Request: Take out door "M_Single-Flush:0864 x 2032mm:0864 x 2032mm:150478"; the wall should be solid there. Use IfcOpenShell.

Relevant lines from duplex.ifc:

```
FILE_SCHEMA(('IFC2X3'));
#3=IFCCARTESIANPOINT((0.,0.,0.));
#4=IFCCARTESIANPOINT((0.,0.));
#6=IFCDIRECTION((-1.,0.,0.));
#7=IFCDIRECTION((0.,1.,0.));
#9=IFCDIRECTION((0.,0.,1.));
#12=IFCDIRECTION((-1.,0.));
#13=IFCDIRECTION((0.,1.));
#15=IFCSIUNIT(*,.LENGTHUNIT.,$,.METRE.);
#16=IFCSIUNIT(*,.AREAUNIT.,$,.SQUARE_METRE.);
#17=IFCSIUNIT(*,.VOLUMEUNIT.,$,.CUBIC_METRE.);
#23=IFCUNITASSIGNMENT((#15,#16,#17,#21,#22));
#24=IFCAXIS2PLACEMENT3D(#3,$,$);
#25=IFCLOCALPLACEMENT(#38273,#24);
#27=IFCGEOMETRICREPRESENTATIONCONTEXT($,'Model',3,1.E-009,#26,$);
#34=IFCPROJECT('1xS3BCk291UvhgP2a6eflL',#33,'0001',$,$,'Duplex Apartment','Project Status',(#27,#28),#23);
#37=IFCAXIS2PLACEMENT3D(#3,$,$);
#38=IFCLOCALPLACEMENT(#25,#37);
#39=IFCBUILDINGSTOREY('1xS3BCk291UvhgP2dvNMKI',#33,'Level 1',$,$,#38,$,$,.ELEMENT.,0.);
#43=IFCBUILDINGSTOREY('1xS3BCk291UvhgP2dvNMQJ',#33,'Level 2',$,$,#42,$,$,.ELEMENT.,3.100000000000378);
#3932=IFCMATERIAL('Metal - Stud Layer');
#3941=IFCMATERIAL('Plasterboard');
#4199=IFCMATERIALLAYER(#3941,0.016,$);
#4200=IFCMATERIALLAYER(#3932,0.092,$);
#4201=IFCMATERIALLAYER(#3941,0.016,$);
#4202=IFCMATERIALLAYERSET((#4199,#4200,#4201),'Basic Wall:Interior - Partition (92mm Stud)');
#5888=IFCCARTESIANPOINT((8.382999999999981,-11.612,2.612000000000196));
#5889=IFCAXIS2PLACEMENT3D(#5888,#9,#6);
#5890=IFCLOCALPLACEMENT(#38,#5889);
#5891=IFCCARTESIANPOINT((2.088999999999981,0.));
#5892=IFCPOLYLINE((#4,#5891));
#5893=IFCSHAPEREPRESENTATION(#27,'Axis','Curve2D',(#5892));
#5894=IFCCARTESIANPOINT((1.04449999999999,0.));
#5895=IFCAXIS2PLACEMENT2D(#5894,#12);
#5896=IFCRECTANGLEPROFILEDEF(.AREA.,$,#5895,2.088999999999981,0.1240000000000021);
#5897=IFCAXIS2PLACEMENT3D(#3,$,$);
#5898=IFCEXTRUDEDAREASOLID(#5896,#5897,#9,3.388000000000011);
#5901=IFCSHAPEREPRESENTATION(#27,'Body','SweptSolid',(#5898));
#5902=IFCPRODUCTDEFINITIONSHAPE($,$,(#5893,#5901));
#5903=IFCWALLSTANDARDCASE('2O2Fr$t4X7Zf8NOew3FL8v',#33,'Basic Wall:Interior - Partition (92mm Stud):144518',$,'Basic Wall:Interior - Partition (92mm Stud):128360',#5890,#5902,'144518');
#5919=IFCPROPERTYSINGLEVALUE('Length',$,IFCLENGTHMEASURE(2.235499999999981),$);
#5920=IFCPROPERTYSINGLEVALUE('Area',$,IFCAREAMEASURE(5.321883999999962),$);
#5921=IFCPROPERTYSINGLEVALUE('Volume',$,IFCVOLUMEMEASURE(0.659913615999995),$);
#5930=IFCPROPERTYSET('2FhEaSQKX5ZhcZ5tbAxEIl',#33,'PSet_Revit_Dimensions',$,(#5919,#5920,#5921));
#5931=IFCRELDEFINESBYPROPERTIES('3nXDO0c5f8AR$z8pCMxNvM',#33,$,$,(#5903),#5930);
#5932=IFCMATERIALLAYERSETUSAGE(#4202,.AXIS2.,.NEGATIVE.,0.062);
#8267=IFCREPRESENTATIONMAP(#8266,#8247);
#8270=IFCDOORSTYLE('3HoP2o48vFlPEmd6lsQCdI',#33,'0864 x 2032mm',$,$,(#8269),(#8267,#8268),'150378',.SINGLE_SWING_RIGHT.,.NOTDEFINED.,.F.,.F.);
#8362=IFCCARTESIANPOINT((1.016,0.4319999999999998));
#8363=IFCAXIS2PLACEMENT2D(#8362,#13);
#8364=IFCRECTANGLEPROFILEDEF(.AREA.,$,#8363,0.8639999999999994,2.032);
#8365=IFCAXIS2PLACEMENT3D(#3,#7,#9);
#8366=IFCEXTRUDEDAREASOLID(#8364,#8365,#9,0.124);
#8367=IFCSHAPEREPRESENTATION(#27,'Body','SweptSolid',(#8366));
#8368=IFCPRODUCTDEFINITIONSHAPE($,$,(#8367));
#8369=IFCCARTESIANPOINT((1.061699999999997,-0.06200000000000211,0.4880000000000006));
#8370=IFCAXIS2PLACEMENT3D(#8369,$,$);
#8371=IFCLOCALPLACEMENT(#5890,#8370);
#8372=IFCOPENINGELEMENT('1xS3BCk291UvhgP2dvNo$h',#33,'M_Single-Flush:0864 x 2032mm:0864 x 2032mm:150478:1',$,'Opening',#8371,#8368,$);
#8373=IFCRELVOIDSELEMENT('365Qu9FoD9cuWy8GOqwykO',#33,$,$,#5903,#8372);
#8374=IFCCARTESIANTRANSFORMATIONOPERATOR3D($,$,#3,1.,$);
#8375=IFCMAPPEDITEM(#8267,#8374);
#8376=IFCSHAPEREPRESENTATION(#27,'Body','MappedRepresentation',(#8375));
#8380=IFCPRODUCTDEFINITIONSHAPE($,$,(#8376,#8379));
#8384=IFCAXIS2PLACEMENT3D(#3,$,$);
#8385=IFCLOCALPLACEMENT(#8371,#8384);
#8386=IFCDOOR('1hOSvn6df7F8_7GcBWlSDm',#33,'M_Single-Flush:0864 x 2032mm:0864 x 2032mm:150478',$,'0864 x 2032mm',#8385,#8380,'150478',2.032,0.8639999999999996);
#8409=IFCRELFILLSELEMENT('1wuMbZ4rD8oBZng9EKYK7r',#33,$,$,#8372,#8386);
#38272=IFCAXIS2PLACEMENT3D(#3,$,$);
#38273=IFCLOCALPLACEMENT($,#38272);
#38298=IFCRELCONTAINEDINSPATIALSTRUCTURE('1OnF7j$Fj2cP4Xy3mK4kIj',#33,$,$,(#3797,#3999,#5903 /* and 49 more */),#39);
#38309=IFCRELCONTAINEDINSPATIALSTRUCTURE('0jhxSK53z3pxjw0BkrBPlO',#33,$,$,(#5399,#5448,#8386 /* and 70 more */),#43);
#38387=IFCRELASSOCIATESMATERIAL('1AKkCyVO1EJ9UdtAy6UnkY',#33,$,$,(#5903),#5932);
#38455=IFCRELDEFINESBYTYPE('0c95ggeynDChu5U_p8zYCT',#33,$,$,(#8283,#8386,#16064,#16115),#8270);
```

```python
import ifcopenshell
import ifcopenshell.api.feature
import ifcopenshell.api.pset
import ifcopenshell.api.root
import ifcopenshell.geom
import ifcopenshell.util.element
import ifcopenshell.util.shape
import ifcopenshell.util.unit

model = ifcopenshell.open("duplex.ifc")
area_scale = ifcopenshell.util.unit.calculate_unit_scale(model, "AREAUNIT")
volume_scale = ifcopenshell.util.unit.calculate_unit_scale(model, "VOLUMEUNIT")
settings = ifcopenshell.geom.settings()


def volume(element):
    """Net volume in cubic metres, openings subtracted."""
    shape = ifcopenshell.geom.create_shape(settings, element)
    return ifcopenshell.util.shape.get_volume(shape.geometry)


door = model.by_id(8386)
opening = door.FillsVoids[0].RelatingOpeningElement
wall = opening.VoidsElements[0].RelatingBuildingElement
before = volume(wall)

ifcopenshell.api.root.remove_product(model, product=door)
ifcopenshell.api.feature.remove_feature(model, feature=opening)

after = volume(wall)
thickness = 0.124  # wall thickness in metres

# Update the wall's stored quantities.
pset = model.by_id(ifcopenshell.util.element.get_pset(wall, "PSet_Revit_Dimensions", should_inherit=False)["id"])
ifcopenshell.api.pset.edit_pset(model, pset=pset, properties={
    "Area": model.create_entity("IfcAreaMeasure", after / thickness / area_scale),
    "Volume": model.create_entity("IfcVolumeMeasure", after / volume_scale),
})

print(f"wall volume {before:.3f} -> {after:.3f} m3")

model.write("duplex_edited.ifc")
```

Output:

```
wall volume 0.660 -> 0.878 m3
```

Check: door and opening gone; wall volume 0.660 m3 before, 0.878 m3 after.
